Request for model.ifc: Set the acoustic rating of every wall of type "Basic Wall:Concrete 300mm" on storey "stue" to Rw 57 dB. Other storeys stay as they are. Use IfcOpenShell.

First a look at what the model holds.

```python
import ifcopenshell
import ifcopenshell.util.element

model = ifcopenshell.open("model.ifc")
print(model.schema)
storey = next(s for s in model.by_type("IfcBuildingStorey") if s.Name == "stue")
walls = [e for e in ifcopenshell.util.element.get_decomposition(storey) if e.is_a("IfcWall")]
seen = {}
for e in walls:
    element_type = ifcopenshell.util.element.get_type(e)
    key = (element_type.Name if element_type != e and element_type else None, ifcopenshell.util.element.get_pset(e, "Pset_WallCommon", "AcousticRating"))
    seen[key] = seen.get(key, 0) + 1
for (name, value), count in sorted(seen.items(), key=str):
    print(count, "x", name, "|", value)
```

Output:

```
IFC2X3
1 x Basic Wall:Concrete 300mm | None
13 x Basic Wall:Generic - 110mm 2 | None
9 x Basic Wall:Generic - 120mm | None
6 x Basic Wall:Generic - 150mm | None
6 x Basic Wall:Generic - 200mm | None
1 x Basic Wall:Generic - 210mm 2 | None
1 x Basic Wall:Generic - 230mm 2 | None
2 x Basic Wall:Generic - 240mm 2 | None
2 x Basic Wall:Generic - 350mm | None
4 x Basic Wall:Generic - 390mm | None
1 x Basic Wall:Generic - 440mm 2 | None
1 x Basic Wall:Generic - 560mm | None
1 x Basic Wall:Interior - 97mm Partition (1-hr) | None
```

```python
import ifcopenshell
import ifcopenshell.api.pset
import ifcopenshell.util.element

model = ifcopenshell.open("model.ifc")

storey = next(s for s in model.by_type("IfcBuildingStorey") if s.Name == "stue")
walls = [e for e in ifcopenshell.util.element.get_decomposition(storey) if e.is_a("IfcWall")]

count = 0
for e in walls:
    element_type = ifcopenshell.util.element.get_type(e)
    if element_type in (None, e) or element_type.Name != "Basic Wall:Concrete 300mm":
        continue
    # add_pset returns the element's existing set when there is one.
    pset = ifcopenshell.api.pset.add_pset(model, product=e, name="Pset_WallCommon")
    ifcopenshell.api.pset.edit_pset(model, pset=pset, properties={"AcousticRating": "Rw 57 dB"})
    count += 1

print(count, "walls updated")

model.write("model_rev.ifc")
```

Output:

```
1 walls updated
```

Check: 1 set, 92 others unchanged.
